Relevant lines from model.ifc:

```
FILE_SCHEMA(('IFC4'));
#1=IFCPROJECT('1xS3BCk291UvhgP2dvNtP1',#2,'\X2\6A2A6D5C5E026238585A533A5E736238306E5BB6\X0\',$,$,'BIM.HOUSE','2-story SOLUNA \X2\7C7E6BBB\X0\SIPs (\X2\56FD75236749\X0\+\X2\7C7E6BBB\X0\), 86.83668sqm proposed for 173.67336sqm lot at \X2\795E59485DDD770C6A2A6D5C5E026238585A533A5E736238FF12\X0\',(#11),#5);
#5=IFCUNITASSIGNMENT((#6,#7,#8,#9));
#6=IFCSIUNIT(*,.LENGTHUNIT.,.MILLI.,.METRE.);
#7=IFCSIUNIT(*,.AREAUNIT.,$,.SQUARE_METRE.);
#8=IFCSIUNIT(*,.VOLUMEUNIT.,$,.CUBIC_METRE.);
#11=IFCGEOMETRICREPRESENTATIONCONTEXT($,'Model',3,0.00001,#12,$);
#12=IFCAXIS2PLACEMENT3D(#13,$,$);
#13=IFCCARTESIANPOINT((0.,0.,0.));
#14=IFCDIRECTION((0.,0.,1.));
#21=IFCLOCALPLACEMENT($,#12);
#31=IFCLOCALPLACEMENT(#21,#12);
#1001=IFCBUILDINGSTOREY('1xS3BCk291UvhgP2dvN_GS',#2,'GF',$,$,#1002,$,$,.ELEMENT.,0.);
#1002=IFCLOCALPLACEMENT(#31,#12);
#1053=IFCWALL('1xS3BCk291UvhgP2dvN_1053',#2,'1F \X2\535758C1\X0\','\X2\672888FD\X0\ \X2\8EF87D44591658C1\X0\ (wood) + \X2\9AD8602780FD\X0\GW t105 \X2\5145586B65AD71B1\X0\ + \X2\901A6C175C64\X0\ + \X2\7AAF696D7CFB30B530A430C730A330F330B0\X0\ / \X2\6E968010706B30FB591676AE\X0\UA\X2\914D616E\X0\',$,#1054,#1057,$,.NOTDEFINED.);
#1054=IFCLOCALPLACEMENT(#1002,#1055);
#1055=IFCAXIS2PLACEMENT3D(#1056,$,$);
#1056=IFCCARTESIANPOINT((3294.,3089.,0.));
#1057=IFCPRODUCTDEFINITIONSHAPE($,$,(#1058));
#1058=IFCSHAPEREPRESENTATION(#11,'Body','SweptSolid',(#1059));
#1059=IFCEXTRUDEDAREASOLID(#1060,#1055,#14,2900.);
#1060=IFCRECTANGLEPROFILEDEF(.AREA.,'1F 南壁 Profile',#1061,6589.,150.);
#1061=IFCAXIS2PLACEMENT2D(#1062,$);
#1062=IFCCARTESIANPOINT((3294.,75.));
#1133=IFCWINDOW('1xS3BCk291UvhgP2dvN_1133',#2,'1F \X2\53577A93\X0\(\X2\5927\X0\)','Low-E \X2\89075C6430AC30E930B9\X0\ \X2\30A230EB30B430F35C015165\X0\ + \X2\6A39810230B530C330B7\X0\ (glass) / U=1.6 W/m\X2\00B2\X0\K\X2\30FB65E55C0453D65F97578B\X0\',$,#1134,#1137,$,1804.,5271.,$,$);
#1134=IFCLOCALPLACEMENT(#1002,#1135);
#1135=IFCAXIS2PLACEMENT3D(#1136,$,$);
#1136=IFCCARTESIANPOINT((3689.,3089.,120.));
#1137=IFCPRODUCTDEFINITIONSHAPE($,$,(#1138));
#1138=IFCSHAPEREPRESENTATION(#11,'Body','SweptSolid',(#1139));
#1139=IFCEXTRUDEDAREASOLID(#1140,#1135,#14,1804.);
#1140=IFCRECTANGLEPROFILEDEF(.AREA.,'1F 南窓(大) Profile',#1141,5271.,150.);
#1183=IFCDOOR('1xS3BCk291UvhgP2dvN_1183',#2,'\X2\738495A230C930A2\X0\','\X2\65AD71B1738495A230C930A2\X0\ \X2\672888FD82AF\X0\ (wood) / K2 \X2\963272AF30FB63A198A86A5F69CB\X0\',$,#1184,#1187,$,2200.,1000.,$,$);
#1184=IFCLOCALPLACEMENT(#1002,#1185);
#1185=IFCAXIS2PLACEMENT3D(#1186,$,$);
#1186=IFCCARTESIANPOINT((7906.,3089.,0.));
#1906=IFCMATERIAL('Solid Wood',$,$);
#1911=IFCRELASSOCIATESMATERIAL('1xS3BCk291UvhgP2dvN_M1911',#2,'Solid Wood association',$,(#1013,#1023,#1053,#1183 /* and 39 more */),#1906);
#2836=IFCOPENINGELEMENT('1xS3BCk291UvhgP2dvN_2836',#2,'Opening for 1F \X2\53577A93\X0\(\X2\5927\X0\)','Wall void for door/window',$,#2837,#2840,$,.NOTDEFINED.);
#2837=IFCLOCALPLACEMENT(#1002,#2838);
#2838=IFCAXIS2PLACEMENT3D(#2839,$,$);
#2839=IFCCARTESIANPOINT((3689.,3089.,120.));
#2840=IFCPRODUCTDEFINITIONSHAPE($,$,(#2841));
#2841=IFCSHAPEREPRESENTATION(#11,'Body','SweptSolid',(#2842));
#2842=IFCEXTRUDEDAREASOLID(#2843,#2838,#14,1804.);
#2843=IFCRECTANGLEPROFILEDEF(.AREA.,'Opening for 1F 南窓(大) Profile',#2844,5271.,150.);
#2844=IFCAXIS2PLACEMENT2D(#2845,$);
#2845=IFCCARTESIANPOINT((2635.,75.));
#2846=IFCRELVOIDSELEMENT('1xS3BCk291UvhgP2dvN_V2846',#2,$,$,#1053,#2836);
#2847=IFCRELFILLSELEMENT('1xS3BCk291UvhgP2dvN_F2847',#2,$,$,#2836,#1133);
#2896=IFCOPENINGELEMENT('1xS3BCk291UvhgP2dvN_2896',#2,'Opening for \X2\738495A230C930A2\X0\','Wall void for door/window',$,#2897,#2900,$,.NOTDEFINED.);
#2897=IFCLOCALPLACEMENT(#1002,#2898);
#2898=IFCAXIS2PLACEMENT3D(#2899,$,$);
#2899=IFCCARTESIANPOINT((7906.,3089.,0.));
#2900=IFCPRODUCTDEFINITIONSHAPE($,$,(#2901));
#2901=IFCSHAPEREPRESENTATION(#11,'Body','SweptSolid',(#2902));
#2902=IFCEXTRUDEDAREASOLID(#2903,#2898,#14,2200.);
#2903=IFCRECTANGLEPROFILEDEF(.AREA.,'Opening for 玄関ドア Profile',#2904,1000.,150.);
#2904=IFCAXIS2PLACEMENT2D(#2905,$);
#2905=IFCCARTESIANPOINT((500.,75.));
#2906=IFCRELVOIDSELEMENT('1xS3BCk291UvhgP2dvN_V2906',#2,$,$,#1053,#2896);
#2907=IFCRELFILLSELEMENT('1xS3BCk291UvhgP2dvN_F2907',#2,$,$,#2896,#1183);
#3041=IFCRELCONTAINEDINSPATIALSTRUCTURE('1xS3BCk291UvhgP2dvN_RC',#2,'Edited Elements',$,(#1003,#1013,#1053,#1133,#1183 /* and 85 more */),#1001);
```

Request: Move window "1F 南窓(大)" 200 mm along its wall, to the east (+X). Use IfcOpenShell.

```python
import ifcopenshell
import ifcopenshell.api.geometry
import ifcopenshell.util.placement

model = ifcopenshell.open("model.ifc")

window = model.by_guid("1xS3BCk291UvhgP2dvN_1133")
opening = window.FillsVoids[0].RelatingOpeningElement
wall = opening.VoidsElements[0].RelatingBuildingElement

wall_matrix = ifcopenshell.util.placement.get_local_placement(wall.ObjectPlacement)
shift = wall_matrix[:3, 0] * 200.0
before = ifcopenshell.util.placement.get_local_placement(window.ObjectPlacement)[:3, 3].copy()

# The window is not placed relative to its opening, so move both.
for product in (opening, window):
    matrix = ifcopenshell.util.placement.get_local_placement(product.ObjectPlacement)
    matrix[:3, 3] += shift
    ifcopenshell.api.geometry.edit_object_placement(model, product=product, matrix=matrix, is_si=False)

after = ifcopenshell.util.placement.get_local_placement(window.ObjectPlacement)[:3, 3]
print("window moved by", (after - before).round(3) + 0.0)

model.write("model-out.ifc")
```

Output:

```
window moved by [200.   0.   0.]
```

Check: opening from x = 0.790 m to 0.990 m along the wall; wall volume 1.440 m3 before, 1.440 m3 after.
